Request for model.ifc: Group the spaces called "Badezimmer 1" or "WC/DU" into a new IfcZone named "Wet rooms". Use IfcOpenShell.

First a look at what the model holds.

```python
import ifcopenshell

model = ifcopenshell.open("model.ifc")
print(model.schema)
seen = {}
for space in model.by_type("IfcSpace"):
    seen[space.LongName] = seen.get(space.LongName, 0) + 1
for name, count in sorted(seen.items(), key=str):
    print(count, "x", name)
print("zones:", [z.Name for z in model.by_type("IfcZone")][:20])
```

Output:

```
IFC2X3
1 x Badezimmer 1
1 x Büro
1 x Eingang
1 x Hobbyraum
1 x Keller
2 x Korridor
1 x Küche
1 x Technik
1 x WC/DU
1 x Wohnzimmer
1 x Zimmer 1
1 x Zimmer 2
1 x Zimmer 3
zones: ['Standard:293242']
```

```python
import ifcopenshell
import ifcopenshell.api.group
import ifcopenshell.api.root

model = ifcopenshell.open("model.ifc")

names = {"Badezimmer 1", "WC/DU"}
spaces = [s for s in model.by_type("IfcSpace") if s.LongName in names]

zone = ifcopenshell.api.root.create_entity(model, ifc_class="IfcZone", name="Wet rooms")
ifcopenshell.api.group.assign_group(model, products=spaces, group=zone)
print(len(spaces), "spaces in", zone.Name)

model.write("model-out.ifc")
```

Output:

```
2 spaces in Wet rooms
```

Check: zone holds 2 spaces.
